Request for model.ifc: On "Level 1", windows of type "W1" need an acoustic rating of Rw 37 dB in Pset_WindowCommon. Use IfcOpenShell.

First a look at what the model holds.

```python
import ifcopenshell
import ifcopenshell.util.element

model = ifcopenshell.open("model.ifc")
print(model.schema)
storey = next(s for s in model.by_type("IfcBuildingStorey") if s.Name == "Level 1")
windows = [e for e in ifcopenshell.util.element.get_decomposition(storey) if e.is_a("IfcWindow")]
seen = {}
for e in windows:
    element_type = ifcopenshell.util.element.get_type(e)
    key = (element_type.Name if element_type != e and element_type else None, ifcopenshell.util.element.get_pset(e, "Pset_WindowCommon", "AcousticRating"))
    seen[key] = seen.get(key, 0) + 1
for (name, value), count in sorted(seen.items(), key=str):
    print(count, "x", name, "|", value)
```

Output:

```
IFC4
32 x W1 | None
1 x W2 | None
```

```python
import ifcopenshell
import ifcopenshell.api.pset
import ifcopenshell.util.element

model = ifcopenshell.open("model.ifc")

storey = next(s for s in model.by_type("IfcBuildingStorey") if s.Name == "Level 1")
windows = [e for e in ifcopenshell.util.element.get_decomposition(storey) if e.is_a("IfcWindow")]

count = 0
for e in windows:
    element_type = ifcopenshell.util.element.get_type(e)
    if element_type in (None, e) or element_type.Name != "W1":
        continue
    # add_pset returns the element's existing set when there is one.
    pset = ifcopenshell.api.pset.add_pset(model, product=e, name="Pset_WindowCommon")
    ifcopenshell.api.pset.edit_pset(model, pset=pset, properties={"AcousticRating": "Rw 37 dB"})
    count += 1

print(count, "windows updated")

model.write("model-out.ifc")
```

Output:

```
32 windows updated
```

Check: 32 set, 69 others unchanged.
